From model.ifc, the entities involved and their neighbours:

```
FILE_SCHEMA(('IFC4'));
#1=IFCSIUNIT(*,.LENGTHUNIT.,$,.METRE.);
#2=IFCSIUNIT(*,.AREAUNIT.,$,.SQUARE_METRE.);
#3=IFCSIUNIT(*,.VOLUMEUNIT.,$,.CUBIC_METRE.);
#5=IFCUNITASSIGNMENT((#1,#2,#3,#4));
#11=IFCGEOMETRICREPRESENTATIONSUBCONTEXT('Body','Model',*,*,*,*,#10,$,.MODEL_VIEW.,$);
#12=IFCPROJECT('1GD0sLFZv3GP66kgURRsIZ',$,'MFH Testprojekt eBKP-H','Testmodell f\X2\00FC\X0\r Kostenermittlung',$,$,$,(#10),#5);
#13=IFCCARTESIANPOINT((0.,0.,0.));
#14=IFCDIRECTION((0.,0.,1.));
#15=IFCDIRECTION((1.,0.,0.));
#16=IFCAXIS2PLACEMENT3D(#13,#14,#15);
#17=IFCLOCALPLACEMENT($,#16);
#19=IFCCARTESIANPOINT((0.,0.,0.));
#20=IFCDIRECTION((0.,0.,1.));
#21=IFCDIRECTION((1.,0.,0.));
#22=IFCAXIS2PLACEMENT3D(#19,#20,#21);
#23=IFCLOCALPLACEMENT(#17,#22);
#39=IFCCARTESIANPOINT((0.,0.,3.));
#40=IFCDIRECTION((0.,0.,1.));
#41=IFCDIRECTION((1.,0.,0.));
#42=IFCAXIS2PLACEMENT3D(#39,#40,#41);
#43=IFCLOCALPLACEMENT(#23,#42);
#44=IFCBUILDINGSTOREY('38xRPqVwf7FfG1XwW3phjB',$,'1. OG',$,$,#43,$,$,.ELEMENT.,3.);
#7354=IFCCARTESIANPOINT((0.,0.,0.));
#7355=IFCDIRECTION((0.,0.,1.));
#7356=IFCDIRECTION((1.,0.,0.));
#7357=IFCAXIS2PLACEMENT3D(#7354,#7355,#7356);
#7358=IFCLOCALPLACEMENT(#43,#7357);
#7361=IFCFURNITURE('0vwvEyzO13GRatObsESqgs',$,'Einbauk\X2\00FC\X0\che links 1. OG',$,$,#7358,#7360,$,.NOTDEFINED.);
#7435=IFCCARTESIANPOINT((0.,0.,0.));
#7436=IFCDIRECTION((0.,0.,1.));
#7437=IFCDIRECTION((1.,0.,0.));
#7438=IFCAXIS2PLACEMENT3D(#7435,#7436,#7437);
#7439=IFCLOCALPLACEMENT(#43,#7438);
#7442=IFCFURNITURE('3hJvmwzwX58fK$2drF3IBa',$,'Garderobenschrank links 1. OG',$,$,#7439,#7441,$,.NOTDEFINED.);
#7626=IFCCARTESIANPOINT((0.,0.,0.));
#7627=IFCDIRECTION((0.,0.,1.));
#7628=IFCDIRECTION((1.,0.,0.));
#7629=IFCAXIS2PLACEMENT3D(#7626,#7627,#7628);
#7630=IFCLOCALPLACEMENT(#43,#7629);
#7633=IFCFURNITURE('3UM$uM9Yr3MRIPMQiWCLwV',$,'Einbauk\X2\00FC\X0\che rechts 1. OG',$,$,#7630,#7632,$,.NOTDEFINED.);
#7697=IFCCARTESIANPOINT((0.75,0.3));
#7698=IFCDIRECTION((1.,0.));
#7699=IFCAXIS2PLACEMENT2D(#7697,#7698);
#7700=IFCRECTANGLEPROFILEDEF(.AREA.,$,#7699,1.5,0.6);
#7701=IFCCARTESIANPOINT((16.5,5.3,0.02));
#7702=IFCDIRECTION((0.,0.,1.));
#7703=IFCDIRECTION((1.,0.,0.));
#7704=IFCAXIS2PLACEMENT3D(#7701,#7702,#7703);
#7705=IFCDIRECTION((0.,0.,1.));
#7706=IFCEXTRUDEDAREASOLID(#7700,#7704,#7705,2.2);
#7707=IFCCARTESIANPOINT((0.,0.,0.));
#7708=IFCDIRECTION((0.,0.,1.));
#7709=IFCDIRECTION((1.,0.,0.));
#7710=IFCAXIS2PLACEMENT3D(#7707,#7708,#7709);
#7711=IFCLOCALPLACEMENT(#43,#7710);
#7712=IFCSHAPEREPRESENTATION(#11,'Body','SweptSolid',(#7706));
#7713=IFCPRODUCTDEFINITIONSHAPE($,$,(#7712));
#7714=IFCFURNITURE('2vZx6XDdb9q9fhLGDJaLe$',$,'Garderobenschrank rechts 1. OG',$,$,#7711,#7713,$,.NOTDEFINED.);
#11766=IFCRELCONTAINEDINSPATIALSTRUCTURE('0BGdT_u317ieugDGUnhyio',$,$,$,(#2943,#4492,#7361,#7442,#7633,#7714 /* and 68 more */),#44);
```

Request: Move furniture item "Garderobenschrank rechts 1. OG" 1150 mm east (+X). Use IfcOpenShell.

```python
import ifcopenshell
import ifcopenshell.api.geometry
import ifcopenshell.util.placement
import ifcopenshell.util.unit

model = ifcopenshell.open("model.ifc")
unit_scale = ifcopenshell.util.unit.calculate_unit_scale(model)

item = model.by_guid("2vZx6XDdb9q9fhLGDJaLe$")
matrix = ifcopenshell.util.placement.get_local_placement(item.ObjectPlacement)
matrix[0, 3] += 1.15 / unit_scale
ifcopenshell.api.geometry.edit_object_placement(model, product=item, matrix=matrix, is_si=False)

print(ifcopenshell.util.placement.get_local_placement(item.ObjectPlacement).round(3) + 0.0)

model.write("model_v2.ifc")
```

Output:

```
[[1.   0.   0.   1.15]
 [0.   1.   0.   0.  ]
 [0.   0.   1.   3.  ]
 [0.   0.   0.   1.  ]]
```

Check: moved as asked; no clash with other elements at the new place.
